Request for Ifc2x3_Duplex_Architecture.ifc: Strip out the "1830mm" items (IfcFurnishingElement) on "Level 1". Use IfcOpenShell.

First a look at what the model holds.

```python
import ifcopenshell
import ifcopenshell.util.element

model = ifcopenshell.open("Ifc2x3_Duplex_Architecture.ifc")
print(model.schema)
storey = next(s for s in model.by_type("IfcBuildingStorey") if s.Name == "Level 1")
furniture = [e for e in ifcopenshell.util.element.get_decomposition(storey) if e.is_a("IfcFurnishingElement")]
seen = {}
for e in furniture:
    element_type = ifcopenshell.util.element.get_type(e)
    name = element_type.Name if element_type not in (None, e) else None
    seen[name] = seen.get(name, 0) + 1
for name, count in sorted(seen.items(), key=str):
    print(count, "x", name)
```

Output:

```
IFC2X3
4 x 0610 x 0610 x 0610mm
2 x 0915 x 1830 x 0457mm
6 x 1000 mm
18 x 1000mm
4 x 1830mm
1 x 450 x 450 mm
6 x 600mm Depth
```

```python
import ifcopenshell
import ifcopenshell.api.root
import ifcopenshell.util.element

model = ifcopenshell.open("Ifc2x3_Duplex_Architecture.ifc")

storey = next(s for s in model.by_type("IfcBuildingStorey") if s.Name == "Level 1")
furniture = [e for e in ifcopenshell.util.element.get_decomposition(storey) if e.is_a("IfcFurnishingElement")]
targets = [e for e in furniture if (t := ifcopenshell.util.element.get_type(e)) not in (None, e) and t.Name == "1830mm"]

for e in targets:
    ifcopenshell.api.root.remove_product(model, product=e)
print(len(targets), "removed")

model.write("Ifc2x3_Duplex_Architecture_updated.ifc")
```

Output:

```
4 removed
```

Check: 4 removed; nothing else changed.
